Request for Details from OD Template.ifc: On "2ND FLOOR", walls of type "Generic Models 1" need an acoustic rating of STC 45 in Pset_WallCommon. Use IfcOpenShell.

First a look at what the model holds.

```python
import ifcopenshell
import ifcopenshell.util.element

model = ifcopenshell.open("Details from OD Template.ifc")
print(model.schema)
storey = next(s for s in model.by_type("IfcBuildingStorey") if s.Name == "2ND FLOOR")
walls = [e for e in ifcopenshell.util.element.get_decomposition(storey) if e.is_a("IfcWall")]
seen = {}
for e in walls:
    element_type = ifcopenshell.util.element.get_type(e)
    key = (element_type.Name if element_type != e and element_type else None, ifcopenshell.util.element.get_pset(e, "Pset_WallCommon", "AcousticRating"))
    seen[key] = seen.get(key, 0) + 1
for (name, value), count in sorted(seen.items(), key=str):
    print(count, "x", name, "|", value)
```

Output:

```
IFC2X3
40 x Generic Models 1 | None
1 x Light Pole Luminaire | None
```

```python
import ifcopenshell
import ifcopenshell.api.pset
import ifcopenshell.util.element

model = ifcopenshell.open("Details from OD Template.ifc")

storey = next(s for s in model.by_type("IfcBuildingStorey") if s.Name == "2ND FLOOR")
walls = [e for e in ifcopenshell.util.element.get_decomposition(storey) if e.is_a("IfcWall")]

count = 0
for e in walls:
    element_type = ifcopenshell.util.element.get_type(e)
    if element_type in (None, e) or element_type.Name != "Generic Models 1":
        continue
    # add_pset returns the element's existing set when there is one.
    pset = ifcopenshell.api.pset.add_pset(model, product=e, name="Pset_WallCommon")
    ifcopenshell.api.pset.edit_pset(model, pset=pset, properties={"AcousticRating": "STC 45"})
    count += 1

print(count, "walls updated")

model.write("Details from OD Template_rev.ifc")
```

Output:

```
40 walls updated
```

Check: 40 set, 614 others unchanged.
